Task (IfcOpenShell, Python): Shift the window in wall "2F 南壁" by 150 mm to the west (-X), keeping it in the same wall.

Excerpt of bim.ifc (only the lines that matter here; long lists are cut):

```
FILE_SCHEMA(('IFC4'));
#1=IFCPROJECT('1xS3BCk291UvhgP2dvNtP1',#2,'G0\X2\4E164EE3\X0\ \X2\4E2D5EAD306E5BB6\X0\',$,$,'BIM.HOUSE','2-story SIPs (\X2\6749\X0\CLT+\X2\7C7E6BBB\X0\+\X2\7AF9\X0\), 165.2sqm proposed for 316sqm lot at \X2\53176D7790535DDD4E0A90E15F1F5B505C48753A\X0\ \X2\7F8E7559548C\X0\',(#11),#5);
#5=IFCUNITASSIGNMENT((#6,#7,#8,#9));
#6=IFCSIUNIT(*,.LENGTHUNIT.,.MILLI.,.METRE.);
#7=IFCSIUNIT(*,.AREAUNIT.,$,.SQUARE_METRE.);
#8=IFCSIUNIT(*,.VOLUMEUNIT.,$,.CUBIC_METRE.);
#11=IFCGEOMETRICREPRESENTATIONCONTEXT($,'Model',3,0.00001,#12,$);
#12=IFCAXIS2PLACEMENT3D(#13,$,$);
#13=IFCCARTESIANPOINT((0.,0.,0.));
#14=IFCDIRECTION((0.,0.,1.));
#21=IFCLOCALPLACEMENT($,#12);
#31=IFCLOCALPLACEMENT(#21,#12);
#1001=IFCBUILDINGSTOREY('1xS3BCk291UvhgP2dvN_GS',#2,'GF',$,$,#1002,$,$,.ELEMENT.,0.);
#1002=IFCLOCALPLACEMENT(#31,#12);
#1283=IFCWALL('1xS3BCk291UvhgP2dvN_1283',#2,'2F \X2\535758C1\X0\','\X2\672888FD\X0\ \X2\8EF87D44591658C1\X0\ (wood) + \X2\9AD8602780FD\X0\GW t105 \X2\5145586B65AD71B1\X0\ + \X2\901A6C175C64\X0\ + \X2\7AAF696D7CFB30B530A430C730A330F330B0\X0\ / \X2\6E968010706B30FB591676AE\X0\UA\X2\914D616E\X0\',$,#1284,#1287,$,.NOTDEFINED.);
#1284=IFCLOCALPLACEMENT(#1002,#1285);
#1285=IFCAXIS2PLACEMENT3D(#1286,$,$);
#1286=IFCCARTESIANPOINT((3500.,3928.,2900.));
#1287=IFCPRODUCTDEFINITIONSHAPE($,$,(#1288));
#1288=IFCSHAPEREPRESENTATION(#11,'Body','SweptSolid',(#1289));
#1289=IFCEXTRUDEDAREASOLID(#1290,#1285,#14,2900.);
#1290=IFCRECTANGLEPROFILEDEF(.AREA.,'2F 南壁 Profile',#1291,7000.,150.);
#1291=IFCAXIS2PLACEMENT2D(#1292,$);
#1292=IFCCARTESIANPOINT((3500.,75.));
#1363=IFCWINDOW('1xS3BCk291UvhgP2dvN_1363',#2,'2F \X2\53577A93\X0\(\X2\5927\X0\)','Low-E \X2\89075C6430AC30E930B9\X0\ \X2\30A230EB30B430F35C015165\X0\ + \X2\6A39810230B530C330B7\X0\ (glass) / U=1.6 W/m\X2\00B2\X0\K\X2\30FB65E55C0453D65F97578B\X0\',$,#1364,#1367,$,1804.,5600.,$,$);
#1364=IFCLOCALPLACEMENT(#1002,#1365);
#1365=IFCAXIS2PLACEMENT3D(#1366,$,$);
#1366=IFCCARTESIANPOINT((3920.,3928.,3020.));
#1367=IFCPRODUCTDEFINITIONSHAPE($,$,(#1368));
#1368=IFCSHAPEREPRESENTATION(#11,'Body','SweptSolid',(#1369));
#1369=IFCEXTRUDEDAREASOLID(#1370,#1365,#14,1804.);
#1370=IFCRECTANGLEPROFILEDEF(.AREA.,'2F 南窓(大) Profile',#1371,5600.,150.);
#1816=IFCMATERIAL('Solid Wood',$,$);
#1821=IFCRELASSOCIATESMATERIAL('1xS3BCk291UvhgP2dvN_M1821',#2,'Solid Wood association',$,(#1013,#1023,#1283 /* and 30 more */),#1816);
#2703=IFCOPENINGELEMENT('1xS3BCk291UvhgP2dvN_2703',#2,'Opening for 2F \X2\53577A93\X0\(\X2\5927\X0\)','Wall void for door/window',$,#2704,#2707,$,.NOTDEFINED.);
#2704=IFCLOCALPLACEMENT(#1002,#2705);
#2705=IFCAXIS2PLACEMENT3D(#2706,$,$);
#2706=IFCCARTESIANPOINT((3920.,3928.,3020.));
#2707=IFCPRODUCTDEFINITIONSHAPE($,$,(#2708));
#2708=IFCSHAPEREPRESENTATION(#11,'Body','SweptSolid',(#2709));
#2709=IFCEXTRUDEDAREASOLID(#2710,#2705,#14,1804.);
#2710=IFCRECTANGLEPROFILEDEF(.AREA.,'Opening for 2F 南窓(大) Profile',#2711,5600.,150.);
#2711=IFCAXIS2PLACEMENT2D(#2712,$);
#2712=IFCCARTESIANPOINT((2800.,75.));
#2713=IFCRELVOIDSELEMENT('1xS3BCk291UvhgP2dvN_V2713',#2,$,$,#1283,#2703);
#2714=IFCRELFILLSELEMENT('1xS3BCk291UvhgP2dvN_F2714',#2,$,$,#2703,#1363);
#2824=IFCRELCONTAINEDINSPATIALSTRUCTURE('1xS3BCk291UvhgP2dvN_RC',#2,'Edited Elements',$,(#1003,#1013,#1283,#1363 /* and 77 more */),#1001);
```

```python
import ifcopenshell
import ifcopenshell.api.geometry
import ifcopenshell.util.placement
import ifcopenshell.util.unit

model = ifcopenshell.open("bim.ifc")
unit_scale = ifcopenshell.util.unit.calculate_unit_scale(model)

window = model.by_guid("1xS3BCk291UvhgP2dvN_1363")
opening = window.FillsVoids[0].RelatingOpeningElement
wall = opening.VoidsElements[0].RelatingBuildingElement

wall_matrix = ifcopenshell.util.placement.get_local_placement(wall.ObjectPlacement)
shift = wall_matrix[:3, 0] * -0.15 / unit_scale
before = ifcopenshell.util.placement.get_local_placement(window.ObjectPlacement)[:3, 3].copy()

# The window is not placed relative to its opening, so move both.
for product in (opening, window):
    matrix = ifcopenshell.util.placement.get_local_placement(product.ObjectPlacement)
    matrix[:3, 3] += shift
    ifcopenshell.api.geometry.edit_object_placement(model, product=product, matrix=matrix, is_si=False)

after = ifcopenshell.util.placement.get_local_placement(window.ObjectPlacement)[:3, 3]
print("window moved by", (after - before).round(3) + 0.0)

model.write("bim_updated.ifc")
```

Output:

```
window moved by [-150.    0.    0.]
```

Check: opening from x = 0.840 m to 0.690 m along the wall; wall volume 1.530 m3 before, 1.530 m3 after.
